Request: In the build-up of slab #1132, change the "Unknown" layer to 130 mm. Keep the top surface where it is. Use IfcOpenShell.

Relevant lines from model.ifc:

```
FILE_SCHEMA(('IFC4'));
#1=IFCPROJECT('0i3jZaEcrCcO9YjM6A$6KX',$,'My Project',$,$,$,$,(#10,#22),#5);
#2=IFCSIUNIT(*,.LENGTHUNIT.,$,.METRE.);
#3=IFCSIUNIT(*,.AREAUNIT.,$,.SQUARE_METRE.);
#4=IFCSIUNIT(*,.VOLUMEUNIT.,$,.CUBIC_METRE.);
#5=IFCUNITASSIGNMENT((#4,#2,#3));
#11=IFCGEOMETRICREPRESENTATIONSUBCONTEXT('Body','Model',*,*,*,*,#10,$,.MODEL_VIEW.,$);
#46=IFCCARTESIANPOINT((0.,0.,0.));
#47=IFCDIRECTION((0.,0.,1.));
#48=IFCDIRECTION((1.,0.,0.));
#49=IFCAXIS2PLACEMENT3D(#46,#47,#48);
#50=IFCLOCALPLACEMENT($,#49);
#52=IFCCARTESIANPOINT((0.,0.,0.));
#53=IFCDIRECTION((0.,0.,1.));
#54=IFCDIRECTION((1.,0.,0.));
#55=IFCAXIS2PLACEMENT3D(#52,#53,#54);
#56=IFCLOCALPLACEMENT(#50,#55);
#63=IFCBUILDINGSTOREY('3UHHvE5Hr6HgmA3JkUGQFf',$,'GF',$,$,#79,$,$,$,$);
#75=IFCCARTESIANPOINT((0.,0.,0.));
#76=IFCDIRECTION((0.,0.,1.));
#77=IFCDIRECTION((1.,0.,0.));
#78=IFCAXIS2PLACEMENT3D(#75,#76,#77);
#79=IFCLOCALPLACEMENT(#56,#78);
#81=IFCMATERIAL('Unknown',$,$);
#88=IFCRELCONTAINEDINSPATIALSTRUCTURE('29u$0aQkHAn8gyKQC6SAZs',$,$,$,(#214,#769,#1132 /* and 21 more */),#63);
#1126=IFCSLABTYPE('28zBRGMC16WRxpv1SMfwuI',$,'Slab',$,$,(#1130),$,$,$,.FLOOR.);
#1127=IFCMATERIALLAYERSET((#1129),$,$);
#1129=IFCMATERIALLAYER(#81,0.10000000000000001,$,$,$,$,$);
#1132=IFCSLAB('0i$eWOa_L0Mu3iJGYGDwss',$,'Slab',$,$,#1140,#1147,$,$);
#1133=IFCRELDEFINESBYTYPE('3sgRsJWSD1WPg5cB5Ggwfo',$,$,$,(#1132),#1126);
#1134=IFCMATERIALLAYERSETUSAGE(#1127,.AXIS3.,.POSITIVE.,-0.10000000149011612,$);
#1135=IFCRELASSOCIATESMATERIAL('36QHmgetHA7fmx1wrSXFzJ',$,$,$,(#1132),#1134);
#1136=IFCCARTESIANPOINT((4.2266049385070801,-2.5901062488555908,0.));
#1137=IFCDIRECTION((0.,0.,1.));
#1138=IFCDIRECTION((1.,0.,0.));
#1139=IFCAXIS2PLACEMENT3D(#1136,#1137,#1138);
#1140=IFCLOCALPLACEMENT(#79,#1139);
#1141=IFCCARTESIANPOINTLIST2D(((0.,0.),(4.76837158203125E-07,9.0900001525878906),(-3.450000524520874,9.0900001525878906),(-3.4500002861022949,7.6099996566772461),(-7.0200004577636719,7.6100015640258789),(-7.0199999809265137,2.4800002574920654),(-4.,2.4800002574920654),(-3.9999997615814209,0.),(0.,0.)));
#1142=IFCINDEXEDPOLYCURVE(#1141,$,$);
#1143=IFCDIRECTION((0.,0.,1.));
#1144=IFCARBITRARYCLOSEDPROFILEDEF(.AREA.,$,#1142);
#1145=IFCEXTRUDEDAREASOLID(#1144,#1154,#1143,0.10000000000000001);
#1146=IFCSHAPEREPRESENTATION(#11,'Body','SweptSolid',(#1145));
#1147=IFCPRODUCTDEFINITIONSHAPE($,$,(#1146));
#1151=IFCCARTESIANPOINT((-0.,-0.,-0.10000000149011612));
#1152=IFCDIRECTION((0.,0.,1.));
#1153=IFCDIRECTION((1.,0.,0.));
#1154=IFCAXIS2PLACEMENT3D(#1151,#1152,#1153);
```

```python
import ifcopenshell
import ifcopenshell.util.element
import ifcopenshell.util.representation
import ifcopenshell.util.unit

model = ifcopenshell.open("model.ifc")
unit_scale = ifcopenshell.util.unit.calculate_unit_scale(model)

layer_set = model.by_id(1127)
layer = next(l for l in layer_set.MaterialLayers if l.Material and l.Material.Name == "Unknown")
change = 0.13 / unit_scale - layer.LayerThickness
layer.LayerThickness += change

# Geometry does not follow the layer set by itself.
slabs = [e for e in ifcopenshell.util.element.get_elements_by_material(model, layer_set) if e.is_a("IfcSlab")]
for slab in sorted(slabs, key=lambda e: e.id()):
    body = ifcopenshell.util.representation.get_representation(slab, "Model", "Body")
    solid = body.Items[0]
    old_depth = solid.Depth
    solid.Depth += change
    # Extruded upwards: lower the start of the extrusion so the top stays.
    x, y, z = solid.Position.Location.Coordinates
    solid.Position.Location = model.createIfcCartesianPoint((x, y, z - change))
    print(slab.id(), f"{old_depth:g} -> {solid.Depth:g}")

# The layers are counted up from the underside, which has moved.
for usage in {ifcopenshell.util.element.get_material(slab) for slab in slabs}:
    usage.OffsetFromReferenceLine -= change

model.write("model_updated.ifc")
```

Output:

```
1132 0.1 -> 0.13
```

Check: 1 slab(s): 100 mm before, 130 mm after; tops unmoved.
